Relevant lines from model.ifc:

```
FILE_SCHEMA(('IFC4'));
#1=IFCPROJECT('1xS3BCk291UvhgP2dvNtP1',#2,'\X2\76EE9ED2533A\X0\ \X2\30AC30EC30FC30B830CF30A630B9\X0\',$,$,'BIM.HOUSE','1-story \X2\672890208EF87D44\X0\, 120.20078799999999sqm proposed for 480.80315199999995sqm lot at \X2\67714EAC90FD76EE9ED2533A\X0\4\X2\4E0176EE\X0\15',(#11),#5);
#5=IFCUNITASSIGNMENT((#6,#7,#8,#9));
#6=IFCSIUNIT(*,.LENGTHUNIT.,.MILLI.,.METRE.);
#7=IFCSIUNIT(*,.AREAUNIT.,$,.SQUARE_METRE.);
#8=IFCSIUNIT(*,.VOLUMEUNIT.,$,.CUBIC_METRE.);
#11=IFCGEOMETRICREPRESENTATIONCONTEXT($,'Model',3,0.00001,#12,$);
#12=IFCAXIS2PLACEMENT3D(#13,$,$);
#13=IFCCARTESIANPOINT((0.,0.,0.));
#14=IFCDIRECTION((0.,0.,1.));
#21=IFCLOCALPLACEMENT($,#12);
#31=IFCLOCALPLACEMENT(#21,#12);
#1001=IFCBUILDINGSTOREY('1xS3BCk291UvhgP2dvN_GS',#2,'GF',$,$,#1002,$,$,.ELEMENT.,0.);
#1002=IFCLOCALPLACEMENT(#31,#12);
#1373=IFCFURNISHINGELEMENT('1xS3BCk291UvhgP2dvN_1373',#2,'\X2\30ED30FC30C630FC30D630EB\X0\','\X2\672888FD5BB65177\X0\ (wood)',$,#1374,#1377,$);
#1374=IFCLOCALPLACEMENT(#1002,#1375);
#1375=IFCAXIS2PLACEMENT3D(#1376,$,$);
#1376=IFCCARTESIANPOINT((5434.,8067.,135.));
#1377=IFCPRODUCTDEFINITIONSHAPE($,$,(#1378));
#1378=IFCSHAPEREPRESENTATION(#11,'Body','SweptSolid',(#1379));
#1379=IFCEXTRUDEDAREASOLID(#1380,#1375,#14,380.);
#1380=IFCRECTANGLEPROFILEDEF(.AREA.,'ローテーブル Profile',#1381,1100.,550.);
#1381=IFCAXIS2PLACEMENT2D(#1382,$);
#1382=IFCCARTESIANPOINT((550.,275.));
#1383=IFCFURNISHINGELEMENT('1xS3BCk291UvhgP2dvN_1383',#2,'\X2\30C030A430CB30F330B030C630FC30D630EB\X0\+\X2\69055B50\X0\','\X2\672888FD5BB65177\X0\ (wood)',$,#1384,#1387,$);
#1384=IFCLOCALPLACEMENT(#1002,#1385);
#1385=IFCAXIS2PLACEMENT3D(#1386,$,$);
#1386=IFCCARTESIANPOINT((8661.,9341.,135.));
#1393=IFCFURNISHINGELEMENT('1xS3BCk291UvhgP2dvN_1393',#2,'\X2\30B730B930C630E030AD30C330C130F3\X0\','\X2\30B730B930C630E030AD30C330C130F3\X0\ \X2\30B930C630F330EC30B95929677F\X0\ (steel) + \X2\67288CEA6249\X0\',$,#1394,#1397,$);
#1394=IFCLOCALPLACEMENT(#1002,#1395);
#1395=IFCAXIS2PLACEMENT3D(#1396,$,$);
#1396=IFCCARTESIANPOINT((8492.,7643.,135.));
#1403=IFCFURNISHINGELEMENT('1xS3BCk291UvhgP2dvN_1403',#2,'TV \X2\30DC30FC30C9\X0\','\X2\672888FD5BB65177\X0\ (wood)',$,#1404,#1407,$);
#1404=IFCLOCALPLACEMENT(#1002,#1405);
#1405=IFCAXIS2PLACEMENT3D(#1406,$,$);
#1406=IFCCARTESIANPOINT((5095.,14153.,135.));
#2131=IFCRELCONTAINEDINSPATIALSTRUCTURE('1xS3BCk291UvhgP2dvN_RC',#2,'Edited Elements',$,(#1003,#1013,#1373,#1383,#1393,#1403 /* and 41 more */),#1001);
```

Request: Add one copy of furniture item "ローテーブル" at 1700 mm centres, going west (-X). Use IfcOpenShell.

```python
import numpy as np
import ifcopenshell
import ifcopenshell.api.geometry
import ifcopenshell.api.root
import ifcopenshell.util.element
import ifcopenshell.util.placement

model = ifcopenshell.open("model.ifc")


def reuse_history(source, copy):
    """copy_class also copies each property set's owner history, people and application; keep the originals."""
    for rel in copy.IsDefinedBy:
        if rel.is_a("IfcRelDefinesByProperties") and (history := rel.RelatingPropertyDefinition.OwnerHistory):
            rel.RelatingPropertyDefinition.OwnerHistory = source.OwnerHistory
            ifcopenshell.util.element.remove_deep2(model, history)


source = model.by_id(1373)
base = ifcopenshell.util.placement.get_local_placement(source.ObjectPlacement)
step = np.array([-1.0, 0.0, 0.0]) * 1700.0

for i in range(1, 2):
    copy = ifcopenshell.api.root.copy_class(model, product=source)
    copy.Representation = ifcopenshell.util.element.copy_deep(
        model, source.Representation, exclude=["IfcGeometricRepresentationContext", "IfcRepresentationMap"]
    )
    reuse_history(source, copy)
    matrix = base.copy()
    matrix[:3, 3] += i * step
    print("added at", matrix[:3, 3].round(3) + 0.0)
    ifcopenshell.api.geometry.edit_object_placement(model, product=copy, matrix=matrix, is_si=False)

model.write("model_rev.ifc")
```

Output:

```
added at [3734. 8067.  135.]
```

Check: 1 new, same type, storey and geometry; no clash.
